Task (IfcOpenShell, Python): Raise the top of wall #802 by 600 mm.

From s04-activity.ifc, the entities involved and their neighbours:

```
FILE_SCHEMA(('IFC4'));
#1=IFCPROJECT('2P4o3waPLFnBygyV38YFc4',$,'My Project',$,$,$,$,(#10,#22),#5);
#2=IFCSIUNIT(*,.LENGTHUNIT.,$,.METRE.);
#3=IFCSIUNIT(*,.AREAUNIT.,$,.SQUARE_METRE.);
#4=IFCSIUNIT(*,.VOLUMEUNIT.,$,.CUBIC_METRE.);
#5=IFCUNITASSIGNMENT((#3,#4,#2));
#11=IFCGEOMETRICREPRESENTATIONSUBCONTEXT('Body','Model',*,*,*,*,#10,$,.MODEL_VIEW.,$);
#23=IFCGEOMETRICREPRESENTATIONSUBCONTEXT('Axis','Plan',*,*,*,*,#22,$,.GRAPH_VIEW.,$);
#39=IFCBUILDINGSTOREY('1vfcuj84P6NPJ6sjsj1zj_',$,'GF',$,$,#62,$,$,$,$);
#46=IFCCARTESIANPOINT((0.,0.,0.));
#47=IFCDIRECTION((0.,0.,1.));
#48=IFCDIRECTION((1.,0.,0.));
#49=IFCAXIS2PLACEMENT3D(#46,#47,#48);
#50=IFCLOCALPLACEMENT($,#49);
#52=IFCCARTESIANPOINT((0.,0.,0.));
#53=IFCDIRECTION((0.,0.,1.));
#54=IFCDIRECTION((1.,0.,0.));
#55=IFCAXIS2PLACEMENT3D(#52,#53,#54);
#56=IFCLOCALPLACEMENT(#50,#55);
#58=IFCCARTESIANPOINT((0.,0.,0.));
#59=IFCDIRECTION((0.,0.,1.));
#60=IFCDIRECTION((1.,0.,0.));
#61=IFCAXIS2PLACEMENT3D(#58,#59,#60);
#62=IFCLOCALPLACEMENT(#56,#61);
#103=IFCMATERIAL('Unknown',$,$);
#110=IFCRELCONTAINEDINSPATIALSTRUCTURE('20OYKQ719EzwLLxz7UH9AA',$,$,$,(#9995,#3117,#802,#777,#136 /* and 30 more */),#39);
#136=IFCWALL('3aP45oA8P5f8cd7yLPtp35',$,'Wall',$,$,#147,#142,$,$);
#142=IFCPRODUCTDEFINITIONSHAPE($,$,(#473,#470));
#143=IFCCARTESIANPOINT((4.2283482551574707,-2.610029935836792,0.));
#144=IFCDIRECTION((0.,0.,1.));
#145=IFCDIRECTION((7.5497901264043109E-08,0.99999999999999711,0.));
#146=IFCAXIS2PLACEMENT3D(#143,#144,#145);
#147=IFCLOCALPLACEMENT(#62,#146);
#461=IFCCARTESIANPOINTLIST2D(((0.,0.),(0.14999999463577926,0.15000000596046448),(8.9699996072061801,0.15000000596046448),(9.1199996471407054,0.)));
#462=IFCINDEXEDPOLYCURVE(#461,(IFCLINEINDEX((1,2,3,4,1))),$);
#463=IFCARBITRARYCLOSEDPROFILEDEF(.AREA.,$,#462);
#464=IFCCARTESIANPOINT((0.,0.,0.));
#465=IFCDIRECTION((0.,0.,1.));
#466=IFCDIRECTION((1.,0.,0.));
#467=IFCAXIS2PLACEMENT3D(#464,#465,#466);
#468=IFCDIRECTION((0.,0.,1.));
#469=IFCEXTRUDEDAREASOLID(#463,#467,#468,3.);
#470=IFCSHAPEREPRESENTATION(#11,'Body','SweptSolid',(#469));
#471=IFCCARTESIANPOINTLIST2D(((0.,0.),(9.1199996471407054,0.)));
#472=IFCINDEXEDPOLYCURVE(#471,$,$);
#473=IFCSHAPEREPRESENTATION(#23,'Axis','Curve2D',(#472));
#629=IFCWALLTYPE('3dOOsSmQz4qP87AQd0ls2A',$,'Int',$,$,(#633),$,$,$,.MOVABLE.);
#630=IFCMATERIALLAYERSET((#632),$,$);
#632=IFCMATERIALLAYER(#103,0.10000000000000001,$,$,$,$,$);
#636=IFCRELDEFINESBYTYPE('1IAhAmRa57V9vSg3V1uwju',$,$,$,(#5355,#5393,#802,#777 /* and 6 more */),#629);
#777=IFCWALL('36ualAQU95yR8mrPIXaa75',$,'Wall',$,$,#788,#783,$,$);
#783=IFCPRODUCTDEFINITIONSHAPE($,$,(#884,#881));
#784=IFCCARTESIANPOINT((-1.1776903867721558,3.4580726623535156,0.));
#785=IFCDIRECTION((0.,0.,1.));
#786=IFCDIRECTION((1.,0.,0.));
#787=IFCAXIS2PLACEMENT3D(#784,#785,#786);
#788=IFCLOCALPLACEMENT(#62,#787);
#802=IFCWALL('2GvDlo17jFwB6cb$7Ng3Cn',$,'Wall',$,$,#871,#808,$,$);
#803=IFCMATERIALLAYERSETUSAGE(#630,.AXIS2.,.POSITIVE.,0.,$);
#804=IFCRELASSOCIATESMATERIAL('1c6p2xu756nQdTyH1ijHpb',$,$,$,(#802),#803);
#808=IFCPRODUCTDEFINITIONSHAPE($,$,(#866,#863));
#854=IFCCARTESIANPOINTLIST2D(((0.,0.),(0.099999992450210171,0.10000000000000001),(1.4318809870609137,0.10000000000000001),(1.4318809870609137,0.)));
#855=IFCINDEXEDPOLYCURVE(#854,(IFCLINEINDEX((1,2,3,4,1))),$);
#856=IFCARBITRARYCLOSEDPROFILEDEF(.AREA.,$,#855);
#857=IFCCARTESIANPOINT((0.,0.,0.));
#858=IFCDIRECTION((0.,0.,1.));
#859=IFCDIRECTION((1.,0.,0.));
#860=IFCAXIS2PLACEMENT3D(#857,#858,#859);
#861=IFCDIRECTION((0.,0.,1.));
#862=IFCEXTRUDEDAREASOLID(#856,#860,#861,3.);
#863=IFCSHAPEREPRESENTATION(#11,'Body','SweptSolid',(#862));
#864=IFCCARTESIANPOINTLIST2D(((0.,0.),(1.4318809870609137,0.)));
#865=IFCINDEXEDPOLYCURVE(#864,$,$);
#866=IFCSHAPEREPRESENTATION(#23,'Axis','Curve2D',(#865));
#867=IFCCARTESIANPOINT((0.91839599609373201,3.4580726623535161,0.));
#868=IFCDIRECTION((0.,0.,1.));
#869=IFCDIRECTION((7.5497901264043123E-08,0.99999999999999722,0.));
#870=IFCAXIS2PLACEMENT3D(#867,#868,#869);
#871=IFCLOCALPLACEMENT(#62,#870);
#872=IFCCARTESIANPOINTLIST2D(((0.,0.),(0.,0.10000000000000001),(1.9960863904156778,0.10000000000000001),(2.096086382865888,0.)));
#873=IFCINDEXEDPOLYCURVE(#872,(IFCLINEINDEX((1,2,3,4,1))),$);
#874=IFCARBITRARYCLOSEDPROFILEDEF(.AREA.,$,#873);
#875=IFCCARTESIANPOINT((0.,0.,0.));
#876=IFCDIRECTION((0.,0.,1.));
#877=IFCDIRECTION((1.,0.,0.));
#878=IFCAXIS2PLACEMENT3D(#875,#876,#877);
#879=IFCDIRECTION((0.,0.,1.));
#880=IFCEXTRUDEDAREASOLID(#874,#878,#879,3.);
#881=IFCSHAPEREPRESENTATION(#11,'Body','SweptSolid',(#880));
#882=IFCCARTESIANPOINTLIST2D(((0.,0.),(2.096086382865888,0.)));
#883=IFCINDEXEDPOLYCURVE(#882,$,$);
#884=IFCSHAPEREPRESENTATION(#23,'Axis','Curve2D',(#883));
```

```python
import ifcopenshell
import ifcopenshell.geom
import ifcopenshell.util.representation
import ifcopenshell.util.shape

model = ifcopenshell.open("s04-activity.ifc")
settings = ifcopenshell.geom.settings()


def volume(element):
    """Net volume in cubic metres, openings subtracted."""
    shape = ifcopenshell.geom.create_shape(settings, element)
    return ifcopenshell.util.shape.get_volume(shape.geometry)


wall = model.by_guid("2GvDlo17jFwB6cb$7Ng3Cn")
before = volume(wall)

body = ifcopenshell.util.representation.get_representation(wall, "Model", "Body")
solid = body.Items[0]
old_height = solid.Depth
solid.Depth += 0.6
after = volume(wall)

print(f"height {old_height:g} -> {solid.Depth:g}, volume {before:.3f} -> {after:.3f} m3")

model.write("s04-activity_edited.ifc")
```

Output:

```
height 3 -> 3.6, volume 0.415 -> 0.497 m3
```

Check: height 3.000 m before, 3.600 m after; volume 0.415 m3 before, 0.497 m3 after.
